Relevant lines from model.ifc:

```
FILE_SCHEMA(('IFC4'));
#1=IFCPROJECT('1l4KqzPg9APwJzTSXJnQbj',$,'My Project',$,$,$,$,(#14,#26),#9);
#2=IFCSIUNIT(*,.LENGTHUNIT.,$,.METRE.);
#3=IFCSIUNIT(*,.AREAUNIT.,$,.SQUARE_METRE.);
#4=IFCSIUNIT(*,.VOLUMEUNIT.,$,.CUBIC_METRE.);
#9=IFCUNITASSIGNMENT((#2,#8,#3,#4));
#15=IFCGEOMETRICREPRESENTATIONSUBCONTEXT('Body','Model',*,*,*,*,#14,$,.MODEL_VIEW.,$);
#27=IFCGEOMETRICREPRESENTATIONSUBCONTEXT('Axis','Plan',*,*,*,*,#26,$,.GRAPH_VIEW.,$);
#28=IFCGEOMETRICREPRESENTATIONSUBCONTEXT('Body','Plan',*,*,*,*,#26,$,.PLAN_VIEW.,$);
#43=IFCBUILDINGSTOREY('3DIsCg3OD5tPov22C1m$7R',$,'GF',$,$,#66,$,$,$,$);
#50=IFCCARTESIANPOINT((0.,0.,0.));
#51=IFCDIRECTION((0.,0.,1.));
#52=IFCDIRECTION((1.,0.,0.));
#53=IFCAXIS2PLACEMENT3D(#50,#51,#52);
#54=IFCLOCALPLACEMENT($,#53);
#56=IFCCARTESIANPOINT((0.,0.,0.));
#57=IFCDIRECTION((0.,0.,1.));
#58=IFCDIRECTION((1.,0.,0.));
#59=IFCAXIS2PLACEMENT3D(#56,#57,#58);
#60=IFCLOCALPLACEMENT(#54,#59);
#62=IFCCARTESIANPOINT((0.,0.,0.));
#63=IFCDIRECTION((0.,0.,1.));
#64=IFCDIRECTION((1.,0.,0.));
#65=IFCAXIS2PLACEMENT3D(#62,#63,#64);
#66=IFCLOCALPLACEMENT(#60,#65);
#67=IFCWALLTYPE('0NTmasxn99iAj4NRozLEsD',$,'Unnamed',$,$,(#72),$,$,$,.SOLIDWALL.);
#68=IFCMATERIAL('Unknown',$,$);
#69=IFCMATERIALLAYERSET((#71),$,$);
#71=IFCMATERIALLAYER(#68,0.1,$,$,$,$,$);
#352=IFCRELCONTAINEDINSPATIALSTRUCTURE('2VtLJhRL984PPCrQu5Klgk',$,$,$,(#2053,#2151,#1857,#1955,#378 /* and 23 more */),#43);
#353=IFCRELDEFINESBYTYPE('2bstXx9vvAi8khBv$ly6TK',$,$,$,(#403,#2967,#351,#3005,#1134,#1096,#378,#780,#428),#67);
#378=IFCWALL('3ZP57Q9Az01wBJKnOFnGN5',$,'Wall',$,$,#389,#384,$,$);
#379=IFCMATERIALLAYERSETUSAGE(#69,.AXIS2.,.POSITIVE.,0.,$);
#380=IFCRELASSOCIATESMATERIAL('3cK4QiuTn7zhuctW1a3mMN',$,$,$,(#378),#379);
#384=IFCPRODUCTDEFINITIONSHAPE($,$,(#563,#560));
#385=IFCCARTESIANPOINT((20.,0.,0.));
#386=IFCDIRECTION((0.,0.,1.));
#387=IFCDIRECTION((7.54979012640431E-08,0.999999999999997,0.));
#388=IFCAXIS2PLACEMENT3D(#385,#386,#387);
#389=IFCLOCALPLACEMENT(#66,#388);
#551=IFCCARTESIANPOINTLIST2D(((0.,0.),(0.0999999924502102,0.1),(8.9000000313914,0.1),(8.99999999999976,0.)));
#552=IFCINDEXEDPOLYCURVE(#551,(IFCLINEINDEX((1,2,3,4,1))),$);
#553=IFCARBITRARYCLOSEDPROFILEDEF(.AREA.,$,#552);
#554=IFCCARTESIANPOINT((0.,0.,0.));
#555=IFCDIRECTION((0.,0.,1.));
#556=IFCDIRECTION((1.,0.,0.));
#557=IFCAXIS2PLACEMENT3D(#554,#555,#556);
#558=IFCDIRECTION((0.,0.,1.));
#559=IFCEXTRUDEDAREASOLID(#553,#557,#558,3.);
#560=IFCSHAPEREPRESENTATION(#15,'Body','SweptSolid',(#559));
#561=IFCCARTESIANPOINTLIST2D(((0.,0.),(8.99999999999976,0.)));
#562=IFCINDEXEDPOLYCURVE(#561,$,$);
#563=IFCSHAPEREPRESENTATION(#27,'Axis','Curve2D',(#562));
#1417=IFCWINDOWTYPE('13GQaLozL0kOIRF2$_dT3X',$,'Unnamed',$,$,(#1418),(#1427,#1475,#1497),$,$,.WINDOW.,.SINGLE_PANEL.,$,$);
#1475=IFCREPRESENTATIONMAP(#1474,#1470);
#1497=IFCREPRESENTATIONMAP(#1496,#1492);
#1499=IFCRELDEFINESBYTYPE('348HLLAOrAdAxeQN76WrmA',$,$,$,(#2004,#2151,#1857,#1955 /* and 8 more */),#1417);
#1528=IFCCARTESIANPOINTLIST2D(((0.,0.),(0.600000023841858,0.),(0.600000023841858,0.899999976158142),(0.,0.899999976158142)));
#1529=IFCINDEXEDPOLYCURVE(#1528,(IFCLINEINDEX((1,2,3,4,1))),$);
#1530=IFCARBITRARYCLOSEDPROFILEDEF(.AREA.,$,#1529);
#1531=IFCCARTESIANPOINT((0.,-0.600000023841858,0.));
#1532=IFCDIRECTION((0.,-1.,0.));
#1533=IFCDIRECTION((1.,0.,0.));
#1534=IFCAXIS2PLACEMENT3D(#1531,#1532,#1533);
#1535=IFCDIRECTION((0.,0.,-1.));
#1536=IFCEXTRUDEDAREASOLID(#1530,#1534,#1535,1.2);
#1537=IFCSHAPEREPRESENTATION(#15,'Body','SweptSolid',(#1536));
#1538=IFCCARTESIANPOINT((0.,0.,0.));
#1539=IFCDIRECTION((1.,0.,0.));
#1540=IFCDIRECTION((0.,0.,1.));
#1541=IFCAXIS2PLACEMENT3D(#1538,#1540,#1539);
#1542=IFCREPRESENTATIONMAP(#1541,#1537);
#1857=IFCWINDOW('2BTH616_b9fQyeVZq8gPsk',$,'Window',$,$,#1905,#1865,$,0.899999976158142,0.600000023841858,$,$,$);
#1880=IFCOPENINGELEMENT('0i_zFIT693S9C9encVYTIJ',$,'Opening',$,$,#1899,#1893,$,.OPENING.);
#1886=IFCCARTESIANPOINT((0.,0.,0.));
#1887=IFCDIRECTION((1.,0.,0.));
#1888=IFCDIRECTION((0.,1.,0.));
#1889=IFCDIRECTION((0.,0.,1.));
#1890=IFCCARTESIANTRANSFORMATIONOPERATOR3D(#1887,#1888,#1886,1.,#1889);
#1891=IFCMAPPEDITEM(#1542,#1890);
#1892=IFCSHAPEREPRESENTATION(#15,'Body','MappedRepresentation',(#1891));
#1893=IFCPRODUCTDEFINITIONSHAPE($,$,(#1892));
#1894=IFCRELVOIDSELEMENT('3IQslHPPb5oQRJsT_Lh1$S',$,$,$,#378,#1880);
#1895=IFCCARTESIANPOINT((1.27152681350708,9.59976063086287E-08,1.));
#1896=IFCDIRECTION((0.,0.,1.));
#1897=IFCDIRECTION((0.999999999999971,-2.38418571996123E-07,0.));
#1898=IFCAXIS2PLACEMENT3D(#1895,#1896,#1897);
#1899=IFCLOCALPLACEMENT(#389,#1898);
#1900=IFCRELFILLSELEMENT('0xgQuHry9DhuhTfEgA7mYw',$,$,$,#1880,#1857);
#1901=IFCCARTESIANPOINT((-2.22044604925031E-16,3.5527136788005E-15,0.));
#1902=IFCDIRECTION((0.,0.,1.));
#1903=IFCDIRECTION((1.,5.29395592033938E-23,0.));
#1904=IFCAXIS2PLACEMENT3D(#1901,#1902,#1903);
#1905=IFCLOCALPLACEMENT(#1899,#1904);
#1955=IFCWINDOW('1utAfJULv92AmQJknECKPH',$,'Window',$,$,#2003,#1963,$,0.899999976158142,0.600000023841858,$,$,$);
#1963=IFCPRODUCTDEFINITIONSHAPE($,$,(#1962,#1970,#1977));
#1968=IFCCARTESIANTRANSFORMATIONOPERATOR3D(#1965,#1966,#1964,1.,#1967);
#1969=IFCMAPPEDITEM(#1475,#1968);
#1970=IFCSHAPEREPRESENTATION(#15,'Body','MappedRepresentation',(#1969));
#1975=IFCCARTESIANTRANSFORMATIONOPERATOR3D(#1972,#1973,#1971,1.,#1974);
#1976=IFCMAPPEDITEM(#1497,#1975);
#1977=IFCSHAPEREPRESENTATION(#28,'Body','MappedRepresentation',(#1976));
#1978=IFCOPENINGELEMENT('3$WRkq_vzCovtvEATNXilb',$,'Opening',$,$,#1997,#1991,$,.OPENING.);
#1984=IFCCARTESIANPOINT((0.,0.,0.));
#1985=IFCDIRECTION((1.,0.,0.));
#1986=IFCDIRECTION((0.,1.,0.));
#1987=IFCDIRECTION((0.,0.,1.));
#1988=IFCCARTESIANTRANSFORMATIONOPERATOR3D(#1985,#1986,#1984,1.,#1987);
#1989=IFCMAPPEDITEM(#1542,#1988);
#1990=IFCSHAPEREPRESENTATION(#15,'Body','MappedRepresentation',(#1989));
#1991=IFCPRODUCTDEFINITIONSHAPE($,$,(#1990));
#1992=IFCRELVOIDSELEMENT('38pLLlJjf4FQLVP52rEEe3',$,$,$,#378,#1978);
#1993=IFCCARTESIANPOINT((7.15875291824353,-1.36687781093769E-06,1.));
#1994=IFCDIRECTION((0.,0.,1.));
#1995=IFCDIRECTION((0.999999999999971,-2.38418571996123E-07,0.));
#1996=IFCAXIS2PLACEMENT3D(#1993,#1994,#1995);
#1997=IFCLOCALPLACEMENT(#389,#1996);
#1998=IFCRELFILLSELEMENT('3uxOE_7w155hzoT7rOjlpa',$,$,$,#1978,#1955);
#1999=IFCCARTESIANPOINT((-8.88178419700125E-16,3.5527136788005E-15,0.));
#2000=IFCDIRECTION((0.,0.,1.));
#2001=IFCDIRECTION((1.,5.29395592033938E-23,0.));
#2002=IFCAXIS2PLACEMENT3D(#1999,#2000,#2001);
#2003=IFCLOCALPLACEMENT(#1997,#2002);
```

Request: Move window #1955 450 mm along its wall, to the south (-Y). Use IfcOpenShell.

```python
import ifcopenshell
import ifcopenshell.api.geometry
import ifcopenshell.util.placement

model = ifcopenshell.open("model.ifc")

window = model.by_guid("1utAfJULv92AmQJknECKPH")
opening = window.FillsVoids[0].RelatingOpeningElement
wall = opening.VoidsElements[0].RelatingBuildingElement

wall_matrix = ifcopenshell.util.placement.get_local_placement(wall.ObjectPlacement)
shift = wall_matrix[:3, 0] * -0.45
before = ifcopenshell.util.placement.get_local_placement(window.ObjectPlacement)[:3, 3].copy()

# The window is placed relative to its opening, so it follows when the opening moves.
matrix = ifcopenshell.util.placement.get_local_placement(opening.ObjectPlacement)
matrix[:3, 3] += shift
ifcopenshell.api.geometry.edit_object_placement(
    model, product=opening, matrix=matrix, is_si=False, should_transform_children=True
)

after = ifcopenshell.util.placement.get_local_placement(window.ObjectPlacement)[:3, 3]
print("window moved by", (after - before).round(3) + 0.0)

model.write("model-out.ifc")
```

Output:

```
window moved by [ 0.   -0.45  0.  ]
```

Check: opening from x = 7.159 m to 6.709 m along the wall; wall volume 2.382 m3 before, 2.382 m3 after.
